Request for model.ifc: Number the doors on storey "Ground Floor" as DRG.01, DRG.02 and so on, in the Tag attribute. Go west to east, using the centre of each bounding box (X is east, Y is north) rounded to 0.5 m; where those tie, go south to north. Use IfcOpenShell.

First a look at what the model holds.

```python
import ifcopenshell
import ifcopenshell.util.element
import ifcopenshell.util.placement

model = ifcopenshell.open("model.ifc")
print(model.schema)
storey = next(s for s in model.by_type("IfcBuildingStorey") if s.Name == "Ground Floor")
doors = [e for e in ifcopenshell.util.element.get_decomposition(storey) if e.is_a("IfcDoor")]
for e in sorted(doors, key=lambda e: e.id()):
    origin = ifcopenshell.util.placement.get_local_placement(e.ObjectPlacement)[:3, 3]
    print(e.id(), e.Tag, e.Name, origin.round(2) + 0.0, sep=" | ")
```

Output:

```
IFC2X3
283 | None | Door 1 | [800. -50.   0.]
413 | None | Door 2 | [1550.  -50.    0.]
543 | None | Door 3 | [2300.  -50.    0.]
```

```python
import ifcopenshell
import ifcopenshell.geom
import ifcopenshell.util.element
import ifcopenshell.util.shape

model = ifcopenshell.open("model.ifc")
settings = ifcopenshell.geom.settings()
settings.set("use-world-coords", True)


def centre(element):
    shape = ifcopenshell.geom.create_shape(settings, element)
    return ifcopenshell.util.shape.get_bbox_centroid(shape.geometry)


storey = next(s for s in model.by_type("IfcBuildingStorey") if s.Name == "Ground Floor")
doors = [e for e in ifcopenshell.util.element.get_decomposition(storey) if e.is_a("IfcDoor")]

# Insertion points can sit at a corner or the storey origin, so sort by the geometry (in metres).
centres = {e: centre(e) for e in doors}
doors.sort(key=lambda e: (round(centres[e][0] / 0.5), centres[e][1]))

for i, e in enumerate(doors, start=1):
    number = f"DRG.{i:02d}"
    e.Tag = number
    print(e.id(), number)

model.write("model_updated.ifc")
```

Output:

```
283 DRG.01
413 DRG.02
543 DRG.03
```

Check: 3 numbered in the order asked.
